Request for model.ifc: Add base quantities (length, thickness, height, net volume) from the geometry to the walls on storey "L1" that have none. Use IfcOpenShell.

First a look at what the model holds.

```python
import ifcopenshell
import ifcopenshell.util.element
import ifcopenshell.util.unit

model = ifcopenshell.open("model.ifc")
print(model.schema)
for unit_type in ("LENGTHUNIT", "AREAUNIT", "VOLUMEUNIT"):
    print(unit_type, ifcopenshell.util.unit.calculate_unit_scale(model, unit_type))
storey = next(s for s in model.by_type("IfcBuildingStorey") if s.Name == "L1")
walls = [e for e in ifcopenshell.util.element.get_decomposition(storey) if e.is_a("IfcWall")]
for e in sorted(walls, key=lambda e: e.id()):
    print(e.id(), e.is_a(), e.Name, list(ifcopenshell.util.element.get_psets(e, qtos_only=True)), sep=" | ")
```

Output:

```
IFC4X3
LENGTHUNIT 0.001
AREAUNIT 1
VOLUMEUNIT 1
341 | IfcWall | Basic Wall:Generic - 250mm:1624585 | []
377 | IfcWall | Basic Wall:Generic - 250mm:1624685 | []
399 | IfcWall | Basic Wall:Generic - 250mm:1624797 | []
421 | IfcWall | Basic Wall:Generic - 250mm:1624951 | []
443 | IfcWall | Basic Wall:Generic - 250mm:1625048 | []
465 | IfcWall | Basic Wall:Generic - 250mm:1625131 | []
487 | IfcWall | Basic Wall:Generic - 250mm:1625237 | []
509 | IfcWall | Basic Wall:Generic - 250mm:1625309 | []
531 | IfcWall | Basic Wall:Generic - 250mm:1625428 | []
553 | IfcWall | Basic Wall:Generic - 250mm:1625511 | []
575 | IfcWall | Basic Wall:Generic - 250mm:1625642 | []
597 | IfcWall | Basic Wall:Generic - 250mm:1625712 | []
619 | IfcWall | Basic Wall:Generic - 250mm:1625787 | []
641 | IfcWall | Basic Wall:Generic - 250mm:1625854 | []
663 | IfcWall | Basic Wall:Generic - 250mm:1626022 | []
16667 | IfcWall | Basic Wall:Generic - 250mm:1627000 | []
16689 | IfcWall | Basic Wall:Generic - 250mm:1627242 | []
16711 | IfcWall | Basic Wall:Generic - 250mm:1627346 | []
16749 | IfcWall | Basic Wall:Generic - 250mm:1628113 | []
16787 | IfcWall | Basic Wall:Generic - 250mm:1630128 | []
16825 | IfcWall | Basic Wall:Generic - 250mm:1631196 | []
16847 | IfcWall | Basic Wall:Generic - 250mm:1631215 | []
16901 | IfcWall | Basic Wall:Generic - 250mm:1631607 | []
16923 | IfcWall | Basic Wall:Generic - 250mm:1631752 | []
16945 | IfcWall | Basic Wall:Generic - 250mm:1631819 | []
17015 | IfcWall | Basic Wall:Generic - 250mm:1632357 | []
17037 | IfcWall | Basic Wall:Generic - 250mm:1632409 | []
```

```python
import ifcopenshell
import ifcopenshell.api.pset
import ifcopenshell.geom
import ifcopenshell.util.element
import ifcopenshell.util.shape
import ifcopenshell.util.unit

model = ifcopenshell.open("model.ifc")
unit_scale = ifcopenshell.util.unit.calculate_unit_scale(model)
volume_scale = ifcopenshell.util.unit.calculate_unit_scale(model, "VOLUMEUNIT")
settings = ifcopenshell.geom.settings()

storey = next(s for s in model.by_type("IfcBuildingStorey") if s.Name == "L1")
walls = [e for e in ifcopenshell.util.element.get_decomposition(storey) if e.is_a("IfcWall")]

for e in sorted(walls, key=lambda e: e.id()):
    if ifcopenshell.util.element.get_psets(e, qtos_only=True, should_inherit=False):
        continue
    # Geometry comes back in metres, in the element's own axes.
    shape = ifcopenshell.geom.create_shape(settings, e)
    values = {
        "Length": ifcopenshell.util.shape.get_x(shape.geometry) / unit_scale,
        "Width": ifcopenshell.util.shape.get_y(shape.geometry) / unit_scale,
        "Height": ifcopenshell.util.shape.get_z(shape.geometry) / unit_scale,
        "NetVolume": ifcopenshell.util.shape.get_volume(shape.geometry) / volume_scale,
    }
    qto = ifcopenshell.api.pset.add_qto(model, product=e, name="Qto_WallBaseQuantities")
    ifcopenshell.api.pset.edit_qto(model, qto=qto, properties=values)
    print(e.id(), {k: round(v, 3) for k, v in values.items()})

model.write("model-out.ifc")
```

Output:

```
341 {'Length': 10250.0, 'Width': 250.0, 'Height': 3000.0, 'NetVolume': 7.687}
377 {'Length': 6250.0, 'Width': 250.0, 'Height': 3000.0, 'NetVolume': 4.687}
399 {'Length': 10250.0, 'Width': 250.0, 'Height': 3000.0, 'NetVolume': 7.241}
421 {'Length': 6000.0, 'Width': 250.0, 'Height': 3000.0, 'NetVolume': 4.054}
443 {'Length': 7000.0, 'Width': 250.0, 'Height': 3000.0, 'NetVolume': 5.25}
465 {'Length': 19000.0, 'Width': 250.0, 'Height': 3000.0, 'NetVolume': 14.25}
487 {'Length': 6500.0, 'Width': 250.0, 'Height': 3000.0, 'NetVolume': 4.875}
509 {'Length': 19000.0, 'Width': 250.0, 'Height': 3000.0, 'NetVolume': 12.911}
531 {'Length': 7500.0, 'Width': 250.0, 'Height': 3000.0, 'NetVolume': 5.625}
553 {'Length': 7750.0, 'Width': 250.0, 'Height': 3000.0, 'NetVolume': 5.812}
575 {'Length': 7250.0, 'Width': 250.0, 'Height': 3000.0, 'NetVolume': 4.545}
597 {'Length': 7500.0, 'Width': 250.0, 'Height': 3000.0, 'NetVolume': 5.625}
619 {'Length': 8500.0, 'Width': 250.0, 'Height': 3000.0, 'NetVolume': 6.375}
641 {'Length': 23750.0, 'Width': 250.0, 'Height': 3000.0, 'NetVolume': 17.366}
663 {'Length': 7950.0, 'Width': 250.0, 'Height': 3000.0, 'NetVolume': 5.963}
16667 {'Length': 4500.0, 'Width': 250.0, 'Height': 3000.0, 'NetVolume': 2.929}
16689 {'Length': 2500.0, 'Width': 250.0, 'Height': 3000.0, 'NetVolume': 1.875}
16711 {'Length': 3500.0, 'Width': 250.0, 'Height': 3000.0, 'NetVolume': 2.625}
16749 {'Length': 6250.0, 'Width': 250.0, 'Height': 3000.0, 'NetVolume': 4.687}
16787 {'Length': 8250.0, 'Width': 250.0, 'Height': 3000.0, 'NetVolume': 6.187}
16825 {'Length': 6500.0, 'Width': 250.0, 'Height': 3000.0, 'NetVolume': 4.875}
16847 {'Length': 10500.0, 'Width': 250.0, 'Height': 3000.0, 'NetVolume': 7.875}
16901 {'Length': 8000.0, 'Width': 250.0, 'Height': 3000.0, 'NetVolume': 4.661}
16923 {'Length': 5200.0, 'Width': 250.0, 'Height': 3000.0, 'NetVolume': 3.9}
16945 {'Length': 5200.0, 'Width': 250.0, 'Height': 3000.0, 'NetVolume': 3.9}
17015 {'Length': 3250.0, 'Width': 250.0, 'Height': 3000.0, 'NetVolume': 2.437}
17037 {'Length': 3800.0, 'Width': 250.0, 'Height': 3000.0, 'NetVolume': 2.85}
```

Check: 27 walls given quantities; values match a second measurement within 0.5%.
